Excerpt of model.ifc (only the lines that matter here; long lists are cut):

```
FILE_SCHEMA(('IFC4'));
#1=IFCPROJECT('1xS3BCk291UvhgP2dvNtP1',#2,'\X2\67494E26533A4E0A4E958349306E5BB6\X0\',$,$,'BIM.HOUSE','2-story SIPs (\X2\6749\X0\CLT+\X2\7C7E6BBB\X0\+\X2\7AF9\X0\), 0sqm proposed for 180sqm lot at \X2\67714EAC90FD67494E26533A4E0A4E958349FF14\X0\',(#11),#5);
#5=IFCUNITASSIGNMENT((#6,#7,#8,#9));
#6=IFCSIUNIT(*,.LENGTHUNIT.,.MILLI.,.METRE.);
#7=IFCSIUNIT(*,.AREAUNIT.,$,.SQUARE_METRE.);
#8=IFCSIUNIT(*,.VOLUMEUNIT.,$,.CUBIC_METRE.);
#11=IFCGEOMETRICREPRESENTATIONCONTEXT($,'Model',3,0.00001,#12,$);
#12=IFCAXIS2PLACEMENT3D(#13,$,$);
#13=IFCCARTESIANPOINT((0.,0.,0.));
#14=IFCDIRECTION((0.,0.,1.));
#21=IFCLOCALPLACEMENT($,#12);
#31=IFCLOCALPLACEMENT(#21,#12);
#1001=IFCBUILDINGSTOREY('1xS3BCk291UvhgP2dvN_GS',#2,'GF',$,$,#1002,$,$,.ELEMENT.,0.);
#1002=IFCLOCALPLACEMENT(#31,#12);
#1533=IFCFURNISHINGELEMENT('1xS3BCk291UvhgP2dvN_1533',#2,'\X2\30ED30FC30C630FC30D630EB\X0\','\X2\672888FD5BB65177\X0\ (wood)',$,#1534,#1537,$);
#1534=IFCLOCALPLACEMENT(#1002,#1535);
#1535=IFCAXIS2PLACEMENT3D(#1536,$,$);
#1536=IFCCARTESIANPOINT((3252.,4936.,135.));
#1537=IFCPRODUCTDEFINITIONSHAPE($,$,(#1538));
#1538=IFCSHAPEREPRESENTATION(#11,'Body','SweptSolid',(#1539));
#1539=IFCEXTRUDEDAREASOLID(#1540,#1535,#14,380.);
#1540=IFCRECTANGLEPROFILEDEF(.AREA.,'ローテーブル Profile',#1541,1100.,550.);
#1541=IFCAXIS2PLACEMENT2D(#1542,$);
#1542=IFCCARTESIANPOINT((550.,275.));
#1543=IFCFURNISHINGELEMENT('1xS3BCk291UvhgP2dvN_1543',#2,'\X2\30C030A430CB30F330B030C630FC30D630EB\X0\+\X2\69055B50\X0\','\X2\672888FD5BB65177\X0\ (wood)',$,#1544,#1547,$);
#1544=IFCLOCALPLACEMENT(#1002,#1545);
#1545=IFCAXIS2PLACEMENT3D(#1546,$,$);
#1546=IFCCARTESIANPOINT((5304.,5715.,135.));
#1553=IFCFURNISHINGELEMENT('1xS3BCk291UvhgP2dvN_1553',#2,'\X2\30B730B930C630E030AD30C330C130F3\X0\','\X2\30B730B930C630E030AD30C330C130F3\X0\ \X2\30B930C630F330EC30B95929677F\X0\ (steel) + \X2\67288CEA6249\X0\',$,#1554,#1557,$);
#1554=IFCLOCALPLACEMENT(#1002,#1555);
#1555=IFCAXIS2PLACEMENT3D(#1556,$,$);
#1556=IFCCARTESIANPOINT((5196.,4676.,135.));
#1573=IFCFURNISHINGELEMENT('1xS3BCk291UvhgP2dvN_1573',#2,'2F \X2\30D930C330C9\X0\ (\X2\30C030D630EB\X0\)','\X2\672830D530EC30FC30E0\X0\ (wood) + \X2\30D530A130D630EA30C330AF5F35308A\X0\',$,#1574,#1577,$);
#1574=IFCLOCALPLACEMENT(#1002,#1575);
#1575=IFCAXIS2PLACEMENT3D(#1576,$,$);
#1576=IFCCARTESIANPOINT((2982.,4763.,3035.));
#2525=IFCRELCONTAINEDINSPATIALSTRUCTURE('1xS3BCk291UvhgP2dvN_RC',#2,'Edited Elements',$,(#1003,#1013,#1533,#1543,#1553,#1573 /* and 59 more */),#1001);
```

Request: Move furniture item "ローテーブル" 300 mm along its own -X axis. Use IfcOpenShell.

```python
import ifcopenshell
import ifcopenshell.api.geometry
import ifcopenshell.util.placement
import ifcopenshell.util.unit

model = ifcopenshell.open("model.ifc")
unit_scale = ifcopenshell.util.unit.calculate_unit_scale(model)

item = model.by_guid("1xS3BCk291UvhgP2dvN_1533")
matrix = ifcopenshell.util.placement.get_local_placement(item.ObjectPlacement)
matrix[:3, 3] -= matrix[:3, 0] * 0.3 / unit_scale
ifcopenshell.api.geometry.edit_object_placement(model, product=item, matrix=matrix, is_si=False)

print(ifcopenshell.util.placement.get_local_placement(item.ObjectPlacement).round(3) + 0.0)

model.write("model_edited.ifc")
```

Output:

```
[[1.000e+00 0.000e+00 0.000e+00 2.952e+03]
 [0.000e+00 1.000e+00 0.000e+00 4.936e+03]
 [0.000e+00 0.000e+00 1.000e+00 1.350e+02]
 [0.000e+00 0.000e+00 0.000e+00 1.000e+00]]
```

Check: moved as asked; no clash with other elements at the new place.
